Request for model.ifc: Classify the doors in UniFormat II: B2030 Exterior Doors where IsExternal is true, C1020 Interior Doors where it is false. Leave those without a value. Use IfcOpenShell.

First a look at what the model holds.

```python
import ifcopenshell
import ifcopenshell.util.element

model = ifcopenshell.open("model.ifc")
print(model.schema)
print("classifications:", [c.Name for c in model.by_type("IfcClassification")])
values = [ifcopenshell.util.element.get_pset(e, "Pset_DoorCommon", "IsExternal") for e in model.by_type("IfcDoor")]
for value in (True, False, None):
    print("IsExternal", value, values.count(value))
```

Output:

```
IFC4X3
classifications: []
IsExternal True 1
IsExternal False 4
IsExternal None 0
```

```python
import ifcopenshell
import ifcopenshell.api.classification
import ifcopenshell.util.element

model = ifcopenshell.open("model.ifc")

system = ifcopenshell.api.classification.add_classification(model, classification="UniFormat II")

doors = model.by_type("IfcDoor")
external = {e: ifcopenshell.util.element.get_pset(e, "Pset_DoorCommon", "IsExternal") for e in doors}
for flag, code, name in ((True, "B2030", "Exterior Doors"), (False, "C1020", "Interior Doors")):
    products = [e for e in doors if external[e] is flag]
    ifcopenshell.api.classification.add_reference(
        model, products=products, classification=system, identification=code, name=name
    )
    print(code, len(products))

model.write("model_v2.ifc")
```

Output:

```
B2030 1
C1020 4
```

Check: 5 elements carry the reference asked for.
